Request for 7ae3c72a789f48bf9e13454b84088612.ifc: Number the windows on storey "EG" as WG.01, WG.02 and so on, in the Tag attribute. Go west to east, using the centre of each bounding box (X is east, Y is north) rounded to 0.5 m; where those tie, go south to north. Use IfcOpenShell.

First a look at what the model holds.

```python
import ifcopenshell
import ifcopenshell.util.element
import ifcopenshell.util.placement

model = ifcopenshell.open("7ae3c72a789f48bf9e13454b84088612.ifc")
print(model.schema)
storey = next(s for s in model.by_type("IfcBuildingStorey") if s.Name == "EG")
windows = [e for e in ifcopenshell.util.element.get_decomposition(storey) if e.is_a("IfcWindow")]
for e in sorted(windows, key=lambda e: e.id()):
    origin = ifcopenshell.util.placement.get_local_placement(e.ObjectPlacement)[:3, 3]
    print(e.id(), e.Tag, e.Name, origin.round(2) + 0.0, sep=" | ")
```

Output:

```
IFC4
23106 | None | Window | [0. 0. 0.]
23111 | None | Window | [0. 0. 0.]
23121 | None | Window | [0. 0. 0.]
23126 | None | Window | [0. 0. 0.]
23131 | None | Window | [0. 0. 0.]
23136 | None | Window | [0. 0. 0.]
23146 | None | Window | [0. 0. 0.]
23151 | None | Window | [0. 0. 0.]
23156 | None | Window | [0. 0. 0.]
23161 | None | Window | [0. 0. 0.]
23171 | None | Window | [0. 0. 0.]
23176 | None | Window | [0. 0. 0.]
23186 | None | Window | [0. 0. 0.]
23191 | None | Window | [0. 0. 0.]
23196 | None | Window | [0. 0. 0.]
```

```python
import ifcopenshell
import ifcopenshell.geom
import ifcopenshell.util.element
import ifcopenshell.util.shape

model = ifcopenshell.open("7ae3c72a789f48bf9e13454b84088612.ifc")
settings = ifcopenshell.geom.settings()
settings.set("use-world-coords", True)


def centre(element):
    shape = ifcopenshell.geom.create_shape(settings, element)
    return ifcopenshell.util.shape.get_bbox_centroid(shape.geometry)


storey = next(s for s in model.by_type("IfcBuildingStorey") if s.Name == "EG")
windows = [e for e in ifcopenshell.util.element.get_decomposition(storey) if e.is_a("IfcWindow")]

# Insertion points can sit at a corner or the storey origin, so sort by the geometry (in metres).
centres = {e: centre(e) for e in windows}
windows.sort(key=lambda e: (round(centres[e][0] / 0.5), centres[e][1]))

for i, e in enumerate(windows, start=1):
    number = f"WG.{i:02d}"
    e.Tag = number
    print(e.id(), number)

model.write("7ae3c72a789f48bf9e13454b84088612_rev.ifc")
```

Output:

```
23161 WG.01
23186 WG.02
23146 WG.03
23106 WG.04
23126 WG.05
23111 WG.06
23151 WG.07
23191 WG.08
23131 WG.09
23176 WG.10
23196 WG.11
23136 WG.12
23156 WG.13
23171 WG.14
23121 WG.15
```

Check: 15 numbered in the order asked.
